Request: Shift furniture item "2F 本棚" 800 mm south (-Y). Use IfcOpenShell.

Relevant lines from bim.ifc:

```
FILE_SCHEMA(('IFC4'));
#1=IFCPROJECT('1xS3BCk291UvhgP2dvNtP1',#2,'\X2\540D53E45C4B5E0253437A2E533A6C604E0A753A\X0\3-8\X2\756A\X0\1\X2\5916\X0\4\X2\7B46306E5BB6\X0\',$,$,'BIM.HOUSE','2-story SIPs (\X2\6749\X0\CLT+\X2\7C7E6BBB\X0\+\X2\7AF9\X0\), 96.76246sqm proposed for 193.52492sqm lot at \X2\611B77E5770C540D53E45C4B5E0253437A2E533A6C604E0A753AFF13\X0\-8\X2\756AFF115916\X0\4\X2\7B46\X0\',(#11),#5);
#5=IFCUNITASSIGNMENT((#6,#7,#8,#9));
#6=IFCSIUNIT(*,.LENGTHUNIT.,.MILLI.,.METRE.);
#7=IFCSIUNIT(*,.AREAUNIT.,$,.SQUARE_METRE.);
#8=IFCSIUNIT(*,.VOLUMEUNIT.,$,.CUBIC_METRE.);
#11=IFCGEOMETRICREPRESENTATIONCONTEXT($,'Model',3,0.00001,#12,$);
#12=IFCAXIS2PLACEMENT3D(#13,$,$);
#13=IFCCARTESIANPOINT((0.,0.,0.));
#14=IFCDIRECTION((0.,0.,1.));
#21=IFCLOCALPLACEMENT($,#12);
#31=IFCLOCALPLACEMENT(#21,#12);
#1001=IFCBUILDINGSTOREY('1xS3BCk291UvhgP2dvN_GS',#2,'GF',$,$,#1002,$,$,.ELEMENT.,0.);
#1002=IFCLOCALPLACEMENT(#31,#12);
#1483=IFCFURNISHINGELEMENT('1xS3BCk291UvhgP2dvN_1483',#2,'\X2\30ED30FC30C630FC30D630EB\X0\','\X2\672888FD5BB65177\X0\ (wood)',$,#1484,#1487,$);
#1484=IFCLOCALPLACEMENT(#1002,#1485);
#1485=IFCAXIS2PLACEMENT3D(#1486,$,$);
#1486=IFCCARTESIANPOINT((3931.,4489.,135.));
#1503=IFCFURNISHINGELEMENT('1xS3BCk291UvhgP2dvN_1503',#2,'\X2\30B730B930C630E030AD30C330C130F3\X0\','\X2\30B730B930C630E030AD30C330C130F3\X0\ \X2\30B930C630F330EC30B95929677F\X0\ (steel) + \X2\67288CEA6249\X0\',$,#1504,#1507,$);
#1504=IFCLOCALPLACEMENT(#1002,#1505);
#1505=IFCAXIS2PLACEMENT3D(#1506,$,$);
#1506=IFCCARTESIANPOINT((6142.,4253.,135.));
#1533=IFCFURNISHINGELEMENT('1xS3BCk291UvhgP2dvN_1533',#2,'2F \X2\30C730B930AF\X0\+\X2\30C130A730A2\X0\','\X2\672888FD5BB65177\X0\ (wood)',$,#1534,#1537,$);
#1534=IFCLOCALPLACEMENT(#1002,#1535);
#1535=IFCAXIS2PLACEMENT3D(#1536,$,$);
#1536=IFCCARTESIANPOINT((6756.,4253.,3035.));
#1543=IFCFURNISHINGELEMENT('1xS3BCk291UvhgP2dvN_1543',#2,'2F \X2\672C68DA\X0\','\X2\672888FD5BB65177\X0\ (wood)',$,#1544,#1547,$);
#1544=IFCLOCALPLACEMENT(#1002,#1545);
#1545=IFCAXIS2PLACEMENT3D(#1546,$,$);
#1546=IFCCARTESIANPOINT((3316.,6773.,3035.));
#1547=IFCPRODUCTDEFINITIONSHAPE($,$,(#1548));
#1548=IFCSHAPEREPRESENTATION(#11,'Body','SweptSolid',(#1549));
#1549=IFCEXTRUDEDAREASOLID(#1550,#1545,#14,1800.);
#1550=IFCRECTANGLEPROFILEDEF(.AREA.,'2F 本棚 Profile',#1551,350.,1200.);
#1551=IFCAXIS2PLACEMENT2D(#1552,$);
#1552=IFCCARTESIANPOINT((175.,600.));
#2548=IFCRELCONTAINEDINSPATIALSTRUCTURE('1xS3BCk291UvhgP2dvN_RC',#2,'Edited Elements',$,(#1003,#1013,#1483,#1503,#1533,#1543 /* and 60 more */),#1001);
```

```python
import ifcopenshell
import ifcopenshell.api.geometry
import ifcopenshell.util.placement

model = ifcopenshell.open("bim.ifc")

item = model.by_guid("1xS3BCk291UvhgP2dvN_1543")
matrix = ifcopenshell.util.placement.get_local_placement(item.ObjectPlacement)
matrix[1, 3] -= 800.0
ifcopenshell.api.geometry.edit_object_placement(model, product=item, matrix=matrix, is_si=False)

print(ifcopenshell.util.placement.get_local_placement(item.ObjectPlacement).round(3) + 0.0)

model.write("bim_v2.ifc")
```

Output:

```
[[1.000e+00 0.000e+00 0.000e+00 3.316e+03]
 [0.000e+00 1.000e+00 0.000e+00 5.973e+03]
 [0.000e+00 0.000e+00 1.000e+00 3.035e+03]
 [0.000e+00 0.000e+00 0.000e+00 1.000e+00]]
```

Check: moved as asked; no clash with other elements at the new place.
